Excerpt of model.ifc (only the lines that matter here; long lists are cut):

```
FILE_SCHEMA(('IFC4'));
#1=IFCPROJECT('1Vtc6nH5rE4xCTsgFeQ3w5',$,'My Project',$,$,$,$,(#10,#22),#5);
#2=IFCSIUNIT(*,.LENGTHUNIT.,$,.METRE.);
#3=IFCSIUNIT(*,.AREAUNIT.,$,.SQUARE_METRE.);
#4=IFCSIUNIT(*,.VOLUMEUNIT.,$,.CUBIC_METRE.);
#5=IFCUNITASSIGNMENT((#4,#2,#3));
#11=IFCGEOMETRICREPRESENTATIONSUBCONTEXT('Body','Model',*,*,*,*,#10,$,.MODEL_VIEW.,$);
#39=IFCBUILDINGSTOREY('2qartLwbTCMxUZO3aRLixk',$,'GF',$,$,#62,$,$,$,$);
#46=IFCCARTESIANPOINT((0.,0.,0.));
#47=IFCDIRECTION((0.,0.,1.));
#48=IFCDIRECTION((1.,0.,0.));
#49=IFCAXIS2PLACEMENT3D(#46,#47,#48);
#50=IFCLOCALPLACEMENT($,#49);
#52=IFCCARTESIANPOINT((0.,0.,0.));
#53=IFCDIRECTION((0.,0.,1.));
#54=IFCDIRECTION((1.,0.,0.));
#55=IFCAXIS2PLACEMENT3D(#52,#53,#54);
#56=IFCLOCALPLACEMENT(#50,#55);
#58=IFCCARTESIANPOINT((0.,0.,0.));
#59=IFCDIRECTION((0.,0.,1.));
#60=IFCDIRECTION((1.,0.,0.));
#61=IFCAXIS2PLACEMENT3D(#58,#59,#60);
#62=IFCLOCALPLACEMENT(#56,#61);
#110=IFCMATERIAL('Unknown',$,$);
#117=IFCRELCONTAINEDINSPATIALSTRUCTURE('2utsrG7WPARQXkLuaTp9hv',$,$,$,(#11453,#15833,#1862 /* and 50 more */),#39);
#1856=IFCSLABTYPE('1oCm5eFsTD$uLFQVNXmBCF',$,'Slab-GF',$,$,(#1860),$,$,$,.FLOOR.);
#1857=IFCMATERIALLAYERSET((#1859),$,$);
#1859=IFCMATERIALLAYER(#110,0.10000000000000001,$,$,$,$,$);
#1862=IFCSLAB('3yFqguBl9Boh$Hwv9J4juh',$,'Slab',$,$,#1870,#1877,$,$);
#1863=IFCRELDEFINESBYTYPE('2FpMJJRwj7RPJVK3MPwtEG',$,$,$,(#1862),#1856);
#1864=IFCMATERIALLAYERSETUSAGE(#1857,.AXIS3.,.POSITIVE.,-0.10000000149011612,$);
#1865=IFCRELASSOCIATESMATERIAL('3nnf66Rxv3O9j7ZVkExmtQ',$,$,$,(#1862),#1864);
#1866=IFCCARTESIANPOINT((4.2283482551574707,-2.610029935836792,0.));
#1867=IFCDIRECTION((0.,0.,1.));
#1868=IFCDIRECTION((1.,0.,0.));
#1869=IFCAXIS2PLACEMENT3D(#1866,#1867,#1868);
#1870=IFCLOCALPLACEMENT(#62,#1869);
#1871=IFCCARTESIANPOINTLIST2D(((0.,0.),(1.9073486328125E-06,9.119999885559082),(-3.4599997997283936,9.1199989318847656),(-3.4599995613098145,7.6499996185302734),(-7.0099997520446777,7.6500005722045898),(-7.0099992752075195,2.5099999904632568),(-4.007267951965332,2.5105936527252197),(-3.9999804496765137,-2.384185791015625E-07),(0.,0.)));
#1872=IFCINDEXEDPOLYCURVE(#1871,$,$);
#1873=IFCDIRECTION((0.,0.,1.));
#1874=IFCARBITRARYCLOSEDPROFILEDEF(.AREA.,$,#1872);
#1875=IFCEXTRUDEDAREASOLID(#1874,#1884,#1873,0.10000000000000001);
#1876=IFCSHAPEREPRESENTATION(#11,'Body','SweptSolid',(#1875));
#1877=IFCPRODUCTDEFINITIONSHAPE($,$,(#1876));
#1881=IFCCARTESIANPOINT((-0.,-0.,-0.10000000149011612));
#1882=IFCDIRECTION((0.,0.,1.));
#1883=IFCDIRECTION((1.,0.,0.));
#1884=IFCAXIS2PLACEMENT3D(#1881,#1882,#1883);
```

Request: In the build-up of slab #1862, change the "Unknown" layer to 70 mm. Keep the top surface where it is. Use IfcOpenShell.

```python
import ifcopenshell
import ifcopenshell.util.element
import ifcopenshell.util.representation
import ifcopenshell.util.unit

model = ifcopenshell.open("model.ifc")
unit_scale = ifcopenshell.util.unit.calculate_unit_scale(model)

layer_set = model.by_id(1857)
layer = next(l for l in layer_set.MaterialLayers if l.Material and l.Material.Name == "Unknown")
change = 0.07 / unit_scale - layer.LayerThickness
layer.LayerThickness += change

# Geometry does not follow the layer set by itself.
slabs = [e for e in ifcopenshell.util.element.get_elements_by_material(model, layer_set) if e.is_a("IfcSlab")]
for slab in sorted(slabs, key=lambda e: e.id()):
    body = ifcopenshell.util.representation.get_representation(slab, "Model", "Body")
    solid = body.Items[0]
    old_depth = solid.Depth
    solid.Depth += change
    # Extruded upwards: lower the start of the extrusion so the top stays.
    x, y, z = solid.Position.Location.Coordinates
    solid.Position.Location = model.createIfcCartesianPoint((x, y, z - change))
    print(slab.id(), f"{old_depth:g} -> {solid.Depth:g}")

# The layers are counted up from the underside, which has moved.
for usage in {ifcopenshell.util.element.get_material(slab) for slab in slabs}:
    usage.OffsetFromReferenceLine -= change

model.write("model-out.ifc")
```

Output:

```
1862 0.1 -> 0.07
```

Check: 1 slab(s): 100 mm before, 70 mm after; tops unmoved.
